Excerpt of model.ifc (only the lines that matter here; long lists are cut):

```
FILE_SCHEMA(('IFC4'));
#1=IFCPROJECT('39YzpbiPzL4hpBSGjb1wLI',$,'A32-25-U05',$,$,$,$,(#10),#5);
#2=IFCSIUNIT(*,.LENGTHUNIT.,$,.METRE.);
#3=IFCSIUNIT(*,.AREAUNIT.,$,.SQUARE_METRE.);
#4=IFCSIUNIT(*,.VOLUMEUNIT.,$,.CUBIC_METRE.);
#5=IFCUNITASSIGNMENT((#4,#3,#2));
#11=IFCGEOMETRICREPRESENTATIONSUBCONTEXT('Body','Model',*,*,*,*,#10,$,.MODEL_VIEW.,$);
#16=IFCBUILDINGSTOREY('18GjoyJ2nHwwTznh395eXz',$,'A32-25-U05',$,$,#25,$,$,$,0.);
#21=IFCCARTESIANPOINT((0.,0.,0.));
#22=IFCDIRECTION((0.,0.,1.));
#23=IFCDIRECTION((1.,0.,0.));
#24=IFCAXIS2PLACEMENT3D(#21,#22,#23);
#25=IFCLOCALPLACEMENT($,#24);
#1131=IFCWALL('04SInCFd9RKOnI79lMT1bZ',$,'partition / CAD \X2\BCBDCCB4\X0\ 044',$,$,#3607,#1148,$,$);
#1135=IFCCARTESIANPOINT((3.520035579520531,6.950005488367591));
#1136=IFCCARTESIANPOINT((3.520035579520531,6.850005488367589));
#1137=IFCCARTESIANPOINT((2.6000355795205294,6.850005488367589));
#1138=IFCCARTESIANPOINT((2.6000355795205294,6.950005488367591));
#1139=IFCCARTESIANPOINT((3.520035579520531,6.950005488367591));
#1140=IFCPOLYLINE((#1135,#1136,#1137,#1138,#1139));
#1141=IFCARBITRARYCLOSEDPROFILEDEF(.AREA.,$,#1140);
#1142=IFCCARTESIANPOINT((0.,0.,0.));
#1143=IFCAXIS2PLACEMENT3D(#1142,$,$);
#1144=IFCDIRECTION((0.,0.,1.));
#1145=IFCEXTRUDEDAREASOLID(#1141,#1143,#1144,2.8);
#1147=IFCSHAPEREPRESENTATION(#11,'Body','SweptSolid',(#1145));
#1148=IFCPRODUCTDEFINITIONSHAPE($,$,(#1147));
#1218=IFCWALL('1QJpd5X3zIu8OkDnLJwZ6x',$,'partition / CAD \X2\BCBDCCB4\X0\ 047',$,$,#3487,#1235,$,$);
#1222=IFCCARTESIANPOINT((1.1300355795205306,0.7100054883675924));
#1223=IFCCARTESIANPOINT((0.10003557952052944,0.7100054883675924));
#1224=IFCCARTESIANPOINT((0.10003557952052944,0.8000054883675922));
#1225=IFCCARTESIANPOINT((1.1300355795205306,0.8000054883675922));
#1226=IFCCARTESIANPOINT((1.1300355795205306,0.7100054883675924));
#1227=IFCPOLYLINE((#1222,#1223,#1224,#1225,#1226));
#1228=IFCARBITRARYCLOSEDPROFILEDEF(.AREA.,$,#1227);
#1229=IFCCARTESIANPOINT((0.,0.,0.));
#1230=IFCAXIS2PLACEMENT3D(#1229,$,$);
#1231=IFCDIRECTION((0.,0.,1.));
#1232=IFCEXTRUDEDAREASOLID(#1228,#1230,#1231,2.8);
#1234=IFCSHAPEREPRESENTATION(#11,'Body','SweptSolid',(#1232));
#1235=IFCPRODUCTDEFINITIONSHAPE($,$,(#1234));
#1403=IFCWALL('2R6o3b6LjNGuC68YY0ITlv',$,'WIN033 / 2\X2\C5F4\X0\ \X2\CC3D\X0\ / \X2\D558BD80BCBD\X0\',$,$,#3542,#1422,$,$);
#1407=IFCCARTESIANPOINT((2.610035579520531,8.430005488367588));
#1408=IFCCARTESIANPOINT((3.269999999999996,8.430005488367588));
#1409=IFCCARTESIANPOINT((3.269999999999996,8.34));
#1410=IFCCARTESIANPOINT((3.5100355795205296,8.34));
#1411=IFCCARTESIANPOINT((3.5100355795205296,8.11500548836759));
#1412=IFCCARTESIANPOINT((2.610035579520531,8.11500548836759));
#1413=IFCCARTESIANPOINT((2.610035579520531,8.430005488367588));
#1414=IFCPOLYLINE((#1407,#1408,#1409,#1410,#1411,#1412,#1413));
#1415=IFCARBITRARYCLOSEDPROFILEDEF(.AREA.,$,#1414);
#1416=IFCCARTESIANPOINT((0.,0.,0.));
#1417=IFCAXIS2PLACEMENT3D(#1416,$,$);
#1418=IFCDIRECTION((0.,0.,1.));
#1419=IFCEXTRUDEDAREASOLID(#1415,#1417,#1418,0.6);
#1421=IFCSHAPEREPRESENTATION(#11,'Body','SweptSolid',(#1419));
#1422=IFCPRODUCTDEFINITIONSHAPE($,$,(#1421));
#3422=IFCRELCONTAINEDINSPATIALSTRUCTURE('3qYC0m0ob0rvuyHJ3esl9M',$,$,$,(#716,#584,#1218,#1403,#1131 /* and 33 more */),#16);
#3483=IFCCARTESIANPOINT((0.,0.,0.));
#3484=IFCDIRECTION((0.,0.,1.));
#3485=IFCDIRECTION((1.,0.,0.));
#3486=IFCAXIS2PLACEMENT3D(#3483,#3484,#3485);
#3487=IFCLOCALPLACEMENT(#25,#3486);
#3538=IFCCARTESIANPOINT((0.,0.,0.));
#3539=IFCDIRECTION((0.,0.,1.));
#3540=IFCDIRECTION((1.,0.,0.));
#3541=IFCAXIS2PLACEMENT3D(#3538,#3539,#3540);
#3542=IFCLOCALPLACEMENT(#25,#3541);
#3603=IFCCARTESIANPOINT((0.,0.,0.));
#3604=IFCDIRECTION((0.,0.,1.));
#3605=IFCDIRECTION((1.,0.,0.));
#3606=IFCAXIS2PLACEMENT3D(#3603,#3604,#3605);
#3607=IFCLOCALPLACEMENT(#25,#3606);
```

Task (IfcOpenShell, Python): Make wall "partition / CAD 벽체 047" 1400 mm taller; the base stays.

```python
import ifcopenshell
import ifcopenshell.geom
import ifcopenshell.util.representation
import ifcopenshell.util.shape
import ifcopenshell.util.unit

model = ifcopenshell.open("model.ifc")
unit_scale = ifcopenshell.util.unit.calculate_unit_scale(model)
settings = ifcopenshell.geom.settings()


def volume(element):
    """Net volume in cubic metres, openings subtracted."""
    shape = ifcopenshell.geom.create_shape(settings, element)
    return ifcopenshell.util.shape.get_volume(shape.geometry)


wall = model.by_guid("1QJpd5X3zIu8OkDnLJwZ6x")
before = volume(wall)

body = ifcopenshell.util.representation.get_representation(wall, "Model", "Body")
solid = body.Items[0]
old_height = solid.Depth
solid.Depth += 1.4 / unit_scale
after = volume(wall)

print(f"height {old_height:g} -> {solid.Depth:g}, volume {before:.3f} -> {after:.3f} m3")

model.write("model_rev.ifc")
```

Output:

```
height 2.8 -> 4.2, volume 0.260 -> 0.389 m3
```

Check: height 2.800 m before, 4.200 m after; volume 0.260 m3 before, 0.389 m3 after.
